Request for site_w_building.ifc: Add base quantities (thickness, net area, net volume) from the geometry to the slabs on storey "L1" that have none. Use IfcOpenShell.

First a look at what the model holds.

```python
import ifcopenshell
import ifcopenshell.util.element
import ifcopenshell.util.unit

model = ifcopenshell.open("site_w_building.ifc")
print(model.schema)
for unit_type in ("LENGTHUNIT", "AREAUNIT", "VOLUMEUNIT"):
    print(unit_type, ifcopenshell.util.unit.calculate_unit_scale(model, unit_type))
storey = next(s for s in model.by_type("IfcBuildingStorey") if s.Name == "L1")
slabs = [e for e in ifcopenshell.util.element.get_decomposition(storey) if e.is_a("IfcSlab")]
for e in sorted(slabs, key=lambda e: e.id()):
    print(e.id(), e.is_a(), e.Name, list(ifcopenshell.util.element.get_psets(e, qtos_only=True)), sep=" | ")
```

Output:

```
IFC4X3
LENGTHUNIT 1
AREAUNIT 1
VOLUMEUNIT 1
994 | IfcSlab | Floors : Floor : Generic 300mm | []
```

```python
import ifcopenshell
import ifcopenshell.api.pset
import ifcopenshell.geom
import ifcopenshell.util.element
import ifcopenshell.util.shape
import ifcopenshell.util.unit

model = ifcopenshell.open("site_w_building.ifc")
unit_scale = ifcopenshell.util.unit.calculate_unit_scale(model)
area_scale = ifcopenshell.util.unit.calculate_unit_scale(model, "AREAUNIT")
volume_scale = ifcopenshell.util.unit.calculate_unit_scale(model, "VOLUMEUNIT")
settings = ifcopenshell.geom.settings()

storey = next(s for s in model.by_type("IfcBuildingStorey") if s.Name == "L1")
slabs = [e for e in ifcopenshell.util.element.get_decomposition(storey) if e.is_a("IfcSlab")]

for e in sorted(slabs, key=lambda e: e.id()):
    if ifcopenshell.util.element.get_psets(e, qtos_only=True, should_inherit=False):
        continue
    # Geometry comes back in metres, in the element's own axes.
    shape = ifcopenshell.geom.create_shape(settings, e)
    values = {
        "Width": ifcopenshell.util.shape.get_z(shape.geometry) / unit_scale,
        "NetArea": ifcopenshell.util.shape.get_footprint_area(shape.geometry) / area_scale,
        "NetVolume": ifcopenshell.util.shape.get_volume(shape.geometry) / volume_scale,
    }
    qto = ifcopenshell.api.pset.add_qto(model, product=e, name="Qto_SlabBaseQuantities")
    ifcopenshell.api.pset.edit_qto(model, qto=qto, properties=values)
    print(e.id(), {k: round(v, 3) for k, v in values.items()})

model.write("site_w_building_v2.ifc")
```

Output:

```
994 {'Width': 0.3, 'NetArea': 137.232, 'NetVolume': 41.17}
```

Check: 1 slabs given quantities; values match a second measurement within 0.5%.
